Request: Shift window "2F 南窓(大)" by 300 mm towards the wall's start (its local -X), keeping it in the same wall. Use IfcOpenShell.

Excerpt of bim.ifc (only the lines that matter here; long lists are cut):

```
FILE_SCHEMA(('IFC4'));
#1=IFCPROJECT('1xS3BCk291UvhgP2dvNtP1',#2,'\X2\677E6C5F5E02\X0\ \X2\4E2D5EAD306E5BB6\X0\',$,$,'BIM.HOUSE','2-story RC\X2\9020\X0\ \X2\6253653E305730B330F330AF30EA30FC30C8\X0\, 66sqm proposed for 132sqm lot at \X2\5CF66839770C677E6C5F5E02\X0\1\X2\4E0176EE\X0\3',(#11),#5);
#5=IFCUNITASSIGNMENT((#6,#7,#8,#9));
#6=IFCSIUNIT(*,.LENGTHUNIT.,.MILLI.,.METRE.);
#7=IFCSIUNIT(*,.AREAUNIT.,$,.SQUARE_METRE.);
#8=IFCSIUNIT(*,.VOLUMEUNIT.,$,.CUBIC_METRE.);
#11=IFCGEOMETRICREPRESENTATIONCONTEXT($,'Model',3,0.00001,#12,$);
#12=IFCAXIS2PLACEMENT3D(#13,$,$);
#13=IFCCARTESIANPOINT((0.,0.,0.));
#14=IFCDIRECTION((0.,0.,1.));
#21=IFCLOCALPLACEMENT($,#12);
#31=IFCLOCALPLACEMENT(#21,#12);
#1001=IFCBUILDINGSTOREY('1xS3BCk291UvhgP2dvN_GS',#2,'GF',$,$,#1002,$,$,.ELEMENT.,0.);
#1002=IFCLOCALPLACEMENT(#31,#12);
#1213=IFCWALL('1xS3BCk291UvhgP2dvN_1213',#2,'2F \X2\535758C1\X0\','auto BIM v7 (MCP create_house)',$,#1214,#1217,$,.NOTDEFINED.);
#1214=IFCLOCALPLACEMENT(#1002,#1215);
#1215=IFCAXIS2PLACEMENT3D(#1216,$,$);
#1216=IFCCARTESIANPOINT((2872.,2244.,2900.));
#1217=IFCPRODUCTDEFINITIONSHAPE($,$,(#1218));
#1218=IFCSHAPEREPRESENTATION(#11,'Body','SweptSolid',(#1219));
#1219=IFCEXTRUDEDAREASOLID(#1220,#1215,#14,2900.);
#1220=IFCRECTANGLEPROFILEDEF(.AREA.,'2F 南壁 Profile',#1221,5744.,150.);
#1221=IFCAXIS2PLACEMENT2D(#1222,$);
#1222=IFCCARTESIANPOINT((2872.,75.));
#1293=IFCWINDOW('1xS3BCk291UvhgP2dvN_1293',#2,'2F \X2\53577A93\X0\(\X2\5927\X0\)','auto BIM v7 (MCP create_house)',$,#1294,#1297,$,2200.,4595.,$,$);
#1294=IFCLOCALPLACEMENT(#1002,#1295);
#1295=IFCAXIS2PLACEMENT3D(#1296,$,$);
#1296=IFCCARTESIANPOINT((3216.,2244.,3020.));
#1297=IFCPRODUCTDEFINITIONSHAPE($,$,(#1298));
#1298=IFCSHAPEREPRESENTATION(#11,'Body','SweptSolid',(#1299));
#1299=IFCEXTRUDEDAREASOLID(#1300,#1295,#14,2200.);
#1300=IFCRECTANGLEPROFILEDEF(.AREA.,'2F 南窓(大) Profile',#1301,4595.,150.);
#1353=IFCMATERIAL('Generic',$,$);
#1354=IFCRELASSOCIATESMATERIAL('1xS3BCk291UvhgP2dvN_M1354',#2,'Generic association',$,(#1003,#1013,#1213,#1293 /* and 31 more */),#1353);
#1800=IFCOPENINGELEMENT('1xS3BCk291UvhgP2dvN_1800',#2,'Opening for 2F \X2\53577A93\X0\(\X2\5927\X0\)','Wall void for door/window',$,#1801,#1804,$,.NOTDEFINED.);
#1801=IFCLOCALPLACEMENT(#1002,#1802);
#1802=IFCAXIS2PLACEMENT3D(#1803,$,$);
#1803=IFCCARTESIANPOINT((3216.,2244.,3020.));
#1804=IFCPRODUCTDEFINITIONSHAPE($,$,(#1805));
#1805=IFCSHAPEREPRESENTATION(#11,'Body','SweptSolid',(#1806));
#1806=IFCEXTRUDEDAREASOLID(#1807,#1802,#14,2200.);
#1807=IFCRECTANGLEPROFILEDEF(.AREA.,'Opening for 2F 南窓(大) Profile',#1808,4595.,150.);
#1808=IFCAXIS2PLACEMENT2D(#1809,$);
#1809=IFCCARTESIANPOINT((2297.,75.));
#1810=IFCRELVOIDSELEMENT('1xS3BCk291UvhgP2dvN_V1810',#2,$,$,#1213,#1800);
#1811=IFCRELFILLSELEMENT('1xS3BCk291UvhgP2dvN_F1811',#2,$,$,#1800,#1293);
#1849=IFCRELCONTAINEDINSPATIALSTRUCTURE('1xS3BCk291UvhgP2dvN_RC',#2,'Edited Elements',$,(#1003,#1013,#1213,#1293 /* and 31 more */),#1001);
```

```python
import ifcopenshell
import ifcopenshell.api.geometry
import ifcopenshell.util.placement
import ifcopenshell.util.unit

model = ifcopenshell.open("bim.ifc")
unit_scale = ifcopenshell.util.unit.calculate_unit_scale(model)

window = model.by_id(1293)
opening = window.FillsVoids[0].RelatingOpeningElement
wall = opening.VoidsElements[0].RelatingBuildingElement

wall_matrix = ifcopenshell.util.placement.get_local_placement(wall.ObjectPlacement)
shift = wall_matrix[:3, 0] * -0.3 / unit_scale
before = ifcopenshell.util.placement.get_local_placement(window.ObjectPlacement)[:3, 3].copy()

# The window is not placed relative to its opening, so move both.
for product in (opening, window):
    matrix = ifcopenshell.util.placement.get_local_placement(product.ObjectPlacement)
    matrix[:3, 3] += shift
    ifcopenshell.api.geometry.edit_object_placement(model, product=product, matrix=matrix, is_si=False)

after = ifcopenshell.util.placement.get_local_placement(window.ObjectPlacement)[:3, 3]
print("window moved by", (after - before).round(3) + 0.0)

model.write("bim_rev.ifc")
```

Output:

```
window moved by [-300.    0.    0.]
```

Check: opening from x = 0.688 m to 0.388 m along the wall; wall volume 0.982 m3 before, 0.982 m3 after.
